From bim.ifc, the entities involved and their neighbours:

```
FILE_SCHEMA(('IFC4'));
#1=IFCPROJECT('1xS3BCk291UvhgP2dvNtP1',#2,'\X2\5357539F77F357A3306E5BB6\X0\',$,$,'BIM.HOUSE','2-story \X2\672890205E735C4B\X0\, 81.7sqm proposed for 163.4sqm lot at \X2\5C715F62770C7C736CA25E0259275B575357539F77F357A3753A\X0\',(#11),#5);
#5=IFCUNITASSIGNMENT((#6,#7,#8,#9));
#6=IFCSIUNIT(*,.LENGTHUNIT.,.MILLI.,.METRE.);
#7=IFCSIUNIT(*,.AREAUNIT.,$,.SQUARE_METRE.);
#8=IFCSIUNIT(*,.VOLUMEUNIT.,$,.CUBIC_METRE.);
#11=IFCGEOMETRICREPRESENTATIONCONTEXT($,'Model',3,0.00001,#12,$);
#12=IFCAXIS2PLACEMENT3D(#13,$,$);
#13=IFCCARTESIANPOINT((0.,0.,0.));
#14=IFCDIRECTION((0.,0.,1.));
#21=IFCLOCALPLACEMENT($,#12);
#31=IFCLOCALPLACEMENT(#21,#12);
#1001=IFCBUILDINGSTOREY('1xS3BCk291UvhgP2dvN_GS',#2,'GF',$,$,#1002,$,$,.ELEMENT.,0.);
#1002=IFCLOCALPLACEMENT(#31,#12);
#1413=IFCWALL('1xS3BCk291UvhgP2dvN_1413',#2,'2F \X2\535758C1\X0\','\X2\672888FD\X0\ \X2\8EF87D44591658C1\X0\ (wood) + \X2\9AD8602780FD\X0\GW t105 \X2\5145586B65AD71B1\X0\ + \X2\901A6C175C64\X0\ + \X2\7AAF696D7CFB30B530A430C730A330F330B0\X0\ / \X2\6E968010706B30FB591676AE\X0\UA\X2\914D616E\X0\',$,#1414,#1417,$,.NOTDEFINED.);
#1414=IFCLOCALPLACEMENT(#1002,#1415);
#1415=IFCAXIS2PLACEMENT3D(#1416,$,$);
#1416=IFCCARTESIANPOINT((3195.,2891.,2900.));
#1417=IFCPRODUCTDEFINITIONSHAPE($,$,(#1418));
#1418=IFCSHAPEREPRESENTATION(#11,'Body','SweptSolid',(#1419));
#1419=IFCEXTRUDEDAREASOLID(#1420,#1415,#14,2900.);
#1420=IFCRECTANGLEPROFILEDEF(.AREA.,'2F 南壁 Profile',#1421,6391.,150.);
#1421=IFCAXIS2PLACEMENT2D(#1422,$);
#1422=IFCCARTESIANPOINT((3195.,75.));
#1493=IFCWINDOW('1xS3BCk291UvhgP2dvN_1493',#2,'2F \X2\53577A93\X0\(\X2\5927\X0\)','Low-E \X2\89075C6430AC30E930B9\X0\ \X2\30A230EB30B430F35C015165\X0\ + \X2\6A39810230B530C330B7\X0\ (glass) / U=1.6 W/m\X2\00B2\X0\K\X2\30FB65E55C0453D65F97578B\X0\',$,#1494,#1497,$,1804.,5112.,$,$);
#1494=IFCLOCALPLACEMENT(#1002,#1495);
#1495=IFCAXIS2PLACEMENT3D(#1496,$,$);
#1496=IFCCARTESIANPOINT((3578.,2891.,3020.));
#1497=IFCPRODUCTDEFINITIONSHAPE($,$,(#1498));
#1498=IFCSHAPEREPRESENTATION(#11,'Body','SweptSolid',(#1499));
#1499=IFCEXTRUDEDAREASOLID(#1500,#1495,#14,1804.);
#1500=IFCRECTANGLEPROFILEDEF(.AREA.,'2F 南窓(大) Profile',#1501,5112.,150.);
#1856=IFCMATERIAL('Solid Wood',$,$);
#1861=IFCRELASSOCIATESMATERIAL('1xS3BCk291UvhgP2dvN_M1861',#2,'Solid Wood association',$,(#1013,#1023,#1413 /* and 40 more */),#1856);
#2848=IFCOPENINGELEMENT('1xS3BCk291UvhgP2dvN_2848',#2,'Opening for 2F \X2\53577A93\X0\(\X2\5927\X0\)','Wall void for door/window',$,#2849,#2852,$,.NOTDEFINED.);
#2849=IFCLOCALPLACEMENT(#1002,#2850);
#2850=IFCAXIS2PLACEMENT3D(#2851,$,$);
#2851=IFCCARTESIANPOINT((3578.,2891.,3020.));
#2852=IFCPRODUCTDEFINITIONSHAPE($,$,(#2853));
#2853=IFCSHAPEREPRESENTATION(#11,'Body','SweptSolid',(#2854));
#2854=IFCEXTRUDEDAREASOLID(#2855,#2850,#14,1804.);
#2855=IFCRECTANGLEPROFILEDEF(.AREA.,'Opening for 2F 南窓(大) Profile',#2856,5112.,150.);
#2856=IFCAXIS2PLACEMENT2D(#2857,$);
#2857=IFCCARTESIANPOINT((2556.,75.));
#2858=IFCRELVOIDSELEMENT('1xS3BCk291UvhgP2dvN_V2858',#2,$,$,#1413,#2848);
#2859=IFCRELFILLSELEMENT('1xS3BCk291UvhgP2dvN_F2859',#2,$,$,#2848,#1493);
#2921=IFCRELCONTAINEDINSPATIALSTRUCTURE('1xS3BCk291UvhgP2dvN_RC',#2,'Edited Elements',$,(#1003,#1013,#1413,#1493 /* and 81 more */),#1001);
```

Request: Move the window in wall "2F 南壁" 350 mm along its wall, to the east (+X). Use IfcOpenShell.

```python
import ifcopenshell
import ifcopenshell.api.geometry
import ifcopenshell.util.placement
import ifcopenshell.util.unit

model = ifcopenshell.open("bim.ifc")
unit_scale = ifcopenshell.util.unit.calculate_unit_scale(model)

window = model.by_guid("1xS3BCk291UvhgP2dvN_1493")
opening = window.FillsVoids[0].RelatingOpeningElement
wall = opening.VoidsElements[0].RelatingBuildingElement

wall_matrix = ifcopenshell.util.placement.get_local_placement(wall.ObjectPlacement)
shift = wall_matrix[:3, 0] * 0.35 / unit_scale
before = ifcopenshell.util.placement.get_local_placement(window.ObjectPlacement)[:3, 3].copy()

# The window is not placed relative to its opening, so move both.
for product in (opening, window):
    matrix = ifcopenshell.util.placement.get_local_placement(product.ObjectPlacement)
    matrix[:3, 3] += shift
    ifcopenshell.api.geometry.edit_object_placement(model, product=product, matrix=matrix, is_si=False)

after = ifcopenshell.util.placement.get_local_placement(window.ObjectPlacement)[:3, 3]
print("window moved by", (after - before).round(3) + 0.0)

model.write("bim_edited.ifc")
```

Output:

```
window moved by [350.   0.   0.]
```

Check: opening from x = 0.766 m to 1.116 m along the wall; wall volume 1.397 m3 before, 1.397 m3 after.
